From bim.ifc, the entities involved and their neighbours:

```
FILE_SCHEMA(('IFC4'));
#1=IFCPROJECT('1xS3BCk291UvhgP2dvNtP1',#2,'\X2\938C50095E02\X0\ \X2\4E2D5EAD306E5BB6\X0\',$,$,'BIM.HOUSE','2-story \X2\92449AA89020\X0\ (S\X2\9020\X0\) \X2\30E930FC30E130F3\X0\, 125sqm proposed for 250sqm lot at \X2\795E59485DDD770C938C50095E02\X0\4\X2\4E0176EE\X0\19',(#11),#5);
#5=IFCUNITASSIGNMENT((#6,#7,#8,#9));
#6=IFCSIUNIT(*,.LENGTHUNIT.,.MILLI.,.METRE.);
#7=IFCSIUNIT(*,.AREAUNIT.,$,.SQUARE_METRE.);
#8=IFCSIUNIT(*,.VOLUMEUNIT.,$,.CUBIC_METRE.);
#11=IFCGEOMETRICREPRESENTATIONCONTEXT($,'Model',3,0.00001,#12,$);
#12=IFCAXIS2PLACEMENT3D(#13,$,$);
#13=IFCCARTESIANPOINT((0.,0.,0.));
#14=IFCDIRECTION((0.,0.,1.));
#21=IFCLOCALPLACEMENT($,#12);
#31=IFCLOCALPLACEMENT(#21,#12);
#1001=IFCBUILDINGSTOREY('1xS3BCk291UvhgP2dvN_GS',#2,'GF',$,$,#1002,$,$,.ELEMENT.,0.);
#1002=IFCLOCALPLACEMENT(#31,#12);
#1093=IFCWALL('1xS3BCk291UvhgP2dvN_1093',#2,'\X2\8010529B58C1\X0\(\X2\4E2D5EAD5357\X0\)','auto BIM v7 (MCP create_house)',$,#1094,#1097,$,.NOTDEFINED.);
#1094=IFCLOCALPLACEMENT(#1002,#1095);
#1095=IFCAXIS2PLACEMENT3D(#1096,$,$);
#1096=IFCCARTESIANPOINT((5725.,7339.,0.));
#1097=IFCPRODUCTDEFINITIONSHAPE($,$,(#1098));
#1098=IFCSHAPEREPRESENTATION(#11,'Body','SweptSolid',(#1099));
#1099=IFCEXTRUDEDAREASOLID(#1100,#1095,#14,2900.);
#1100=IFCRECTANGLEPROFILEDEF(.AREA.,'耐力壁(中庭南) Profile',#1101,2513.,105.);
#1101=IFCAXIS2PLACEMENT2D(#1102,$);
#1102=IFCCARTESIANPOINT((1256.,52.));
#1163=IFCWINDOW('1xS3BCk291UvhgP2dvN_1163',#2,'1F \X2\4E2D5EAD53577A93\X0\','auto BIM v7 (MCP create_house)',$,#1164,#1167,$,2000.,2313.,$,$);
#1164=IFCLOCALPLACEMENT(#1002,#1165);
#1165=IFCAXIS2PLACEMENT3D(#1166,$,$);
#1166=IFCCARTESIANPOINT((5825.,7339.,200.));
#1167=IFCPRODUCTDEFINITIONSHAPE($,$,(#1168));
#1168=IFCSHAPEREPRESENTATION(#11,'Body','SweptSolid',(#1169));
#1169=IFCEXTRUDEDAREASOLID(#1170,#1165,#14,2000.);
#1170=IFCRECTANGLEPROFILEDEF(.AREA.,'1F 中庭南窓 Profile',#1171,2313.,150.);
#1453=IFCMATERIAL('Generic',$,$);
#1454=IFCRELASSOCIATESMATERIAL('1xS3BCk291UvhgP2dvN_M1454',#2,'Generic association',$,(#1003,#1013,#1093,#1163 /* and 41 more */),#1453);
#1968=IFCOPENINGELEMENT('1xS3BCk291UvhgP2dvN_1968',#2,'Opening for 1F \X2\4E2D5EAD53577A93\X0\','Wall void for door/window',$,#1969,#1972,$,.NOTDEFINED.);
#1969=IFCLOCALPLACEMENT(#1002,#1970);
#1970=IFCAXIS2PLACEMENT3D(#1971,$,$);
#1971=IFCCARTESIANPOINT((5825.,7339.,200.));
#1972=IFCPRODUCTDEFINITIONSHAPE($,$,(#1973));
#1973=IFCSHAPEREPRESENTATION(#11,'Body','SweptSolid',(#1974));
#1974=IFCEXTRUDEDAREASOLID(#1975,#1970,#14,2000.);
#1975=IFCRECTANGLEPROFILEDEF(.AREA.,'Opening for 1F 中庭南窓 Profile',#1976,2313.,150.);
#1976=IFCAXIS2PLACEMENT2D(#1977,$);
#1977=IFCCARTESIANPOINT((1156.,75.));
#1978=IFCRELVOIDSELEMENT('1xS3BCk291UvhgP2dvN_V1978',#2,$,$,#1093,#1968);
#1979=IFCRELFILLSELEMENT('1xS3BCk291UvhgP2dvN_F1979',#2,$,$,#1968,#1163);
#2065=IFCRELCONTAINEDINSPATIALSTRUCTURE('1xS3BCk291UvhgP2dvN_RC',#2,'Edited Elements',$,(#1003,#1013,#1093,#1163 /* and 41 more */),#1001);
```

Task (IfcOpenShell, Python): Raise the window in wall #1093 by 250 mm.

```python
import numpy as np
import ifcopenshell
import ifcopenshell.api.geometry
import ifcopenshell.util.placement
import ifcopenshell.util.unit

model = ifcopenshell.open("bim.ifc")
unit_scale = ifcopenshell.util.unit.calculate_unit_scale(model)

window = model.by_id(1163)
opening = window.FillsVoids[0].RelatingOpeningElement
dz = 0.25 / unit_scale

shift = np.array([0.0, 0.0, dz])
# The window is not placed relative to its opening, so move both.
for product in (opening, window):
    matrix = ifcopenshell.util.placement.get_local_placement(product.ObjectPlacement)
    matrix[:3, 3] += shift
    ifcopenshell.api.geometry.edit_object_placement(model, product=product, matrix=matrix, is_si=False)

print(f"moved by {dz * unit_scale:+.3f} m")

model.write("bim_v2.ifc")
```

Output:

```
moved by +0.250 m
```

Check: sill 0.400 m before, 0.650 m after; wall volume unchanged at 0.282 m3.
